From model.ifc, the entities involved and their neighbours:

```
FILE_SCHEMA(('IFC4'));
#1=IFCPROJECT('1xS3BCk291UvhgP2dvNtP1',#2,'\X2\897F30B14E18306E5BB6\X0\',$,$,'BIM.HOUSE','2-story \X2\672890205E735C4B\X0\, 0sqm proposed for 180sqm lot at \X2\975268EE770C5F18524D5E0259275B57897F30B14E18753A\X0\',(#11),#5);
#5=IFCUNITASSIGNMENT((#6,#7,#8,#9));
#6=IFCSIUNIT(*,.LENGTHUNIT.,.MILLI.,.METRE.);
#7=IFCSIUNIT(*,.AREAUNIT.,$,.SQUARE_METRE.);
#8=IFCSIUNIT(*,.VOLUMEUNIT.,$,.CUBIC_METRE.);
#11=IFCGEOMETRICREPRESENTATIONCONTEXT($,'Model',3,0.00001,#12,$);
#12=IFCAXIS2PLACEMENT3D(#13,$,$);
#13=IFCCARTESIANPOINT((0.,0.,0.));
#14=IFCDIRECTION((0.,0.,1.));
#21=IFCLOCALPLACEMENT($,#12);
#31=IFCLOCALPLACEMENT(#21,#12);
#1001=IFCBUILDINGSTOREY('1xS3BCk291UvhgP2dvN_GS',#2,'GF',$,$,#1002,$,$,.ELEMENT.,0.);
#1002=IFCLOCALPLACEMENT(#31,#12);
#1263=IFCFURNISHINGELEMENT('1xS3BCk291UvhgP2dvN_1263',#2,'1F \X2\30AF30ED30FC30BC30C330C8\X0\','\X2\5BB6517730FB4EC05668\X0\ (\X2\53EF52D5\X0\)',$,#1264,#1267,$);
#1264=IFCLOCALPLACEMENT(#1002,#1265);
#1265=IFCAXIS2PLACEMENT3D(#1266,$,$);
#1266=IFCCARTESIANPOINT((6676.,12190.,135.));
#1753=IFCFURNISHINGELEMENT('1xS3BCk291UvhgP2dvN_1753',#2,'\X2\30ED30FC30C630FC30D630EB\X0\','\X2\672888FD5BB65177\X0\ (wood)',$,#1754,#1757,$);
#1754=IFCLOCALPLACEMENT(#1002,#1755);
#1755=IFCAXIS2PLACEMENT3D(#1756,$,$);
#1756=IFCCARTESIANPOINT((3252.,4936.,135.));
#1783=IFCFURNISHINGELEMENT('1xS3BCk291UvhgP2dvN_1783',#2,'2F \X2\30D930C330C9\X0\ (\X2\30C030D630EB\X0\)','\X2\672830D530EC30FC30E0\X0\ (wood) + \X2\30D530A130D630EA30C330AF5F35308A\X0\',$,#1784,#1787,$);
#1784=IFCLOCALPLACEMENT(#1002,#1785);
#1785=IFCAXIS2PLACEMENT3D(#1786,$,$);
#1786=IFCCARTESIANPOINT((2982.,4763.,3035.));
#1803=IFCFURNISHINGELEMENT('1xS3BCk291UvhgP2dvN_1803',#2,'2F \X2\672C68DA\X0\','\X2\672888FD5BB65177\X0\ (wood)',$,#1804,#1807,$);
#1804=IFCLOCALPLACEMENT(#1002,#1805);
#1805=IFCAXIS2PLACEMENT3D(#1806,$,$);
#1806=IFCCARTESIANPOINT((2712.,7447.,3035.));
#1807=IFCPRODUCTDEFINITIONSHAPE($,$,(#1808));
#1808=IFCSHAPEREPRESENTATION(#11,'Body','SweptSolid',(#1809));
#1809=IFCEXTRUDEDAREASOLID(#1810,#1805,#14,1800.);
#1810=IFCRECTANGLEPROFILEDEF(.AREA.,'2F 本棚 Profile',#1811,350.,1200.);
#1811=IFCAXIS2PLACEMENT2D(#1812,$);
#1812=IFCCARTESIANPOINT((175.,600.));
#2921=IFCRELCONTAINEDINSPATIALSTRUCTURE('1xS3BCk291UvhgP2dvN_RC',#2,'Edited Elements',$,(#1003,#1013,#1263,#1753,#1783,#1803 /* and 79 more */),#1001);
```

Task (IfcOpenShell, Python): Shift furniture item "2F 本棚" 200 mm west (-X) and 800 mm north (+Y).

```python
import ifcopenshell
import ifcopenshell.api.geometry
import ifcopenshell.util.placement
import ifcopenshell.util.unit

model = ifcopenshell.open("model.ifc")
unit_scale = ifcopenshell.util.unit.calculate_unit_scale(model)

item = model.by_guid("1xS3BCk291UvhgP2dvN_1803")
matrix = ifcopenshell.util.placement.get_local_placement(item.ObjectPlacement)
matrix[0, 3] -= 0.2 / unit_scale
matrix[1, 3] += 0.8 / unit_scale
ifcopenshell.api.geometry.edit_object_placement(model, product=item, matrix=matrix, is_si=False)

print(ifcopenshell.util.placement.get_local_placement(item.ObjectPlacement).round(3) + 0.0)

model.write("model_v2.ifc")
```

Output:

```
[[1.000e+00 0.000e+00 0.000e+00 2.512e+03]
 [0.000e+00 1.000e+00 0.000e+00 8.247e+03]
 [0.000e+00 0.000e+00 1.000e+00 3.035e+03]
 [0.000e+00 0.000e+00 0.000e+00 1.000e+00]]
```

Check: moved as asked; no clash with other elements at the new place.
